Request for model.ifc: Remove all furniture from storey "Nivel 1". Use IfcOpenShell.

First a look at what the model holds.

```python
import ifcopenshell
import ifcopenshell.util.element

model = ifcopenshell.open("model.ifc")
print(model.schema)
storey = next(s for s in model.by_type("IfcBuildingStorey") if s.Name == "Nivel 1")
furniture = [e for e in ifcopenshell.util.element.get_decomposition(storey) if e.is_a("IfcFurnishingElement")]
seen = {}
for e in furniture:
    element_type = ifcopenshell.util.element.get_type(e)
    name = element_type.Name if element_type not in (None, e) else None
    seen[name] = seen.get(name, 0) + 1
for name, count in sorted(seen.items(), key=str):
    print(count, "x", name)
```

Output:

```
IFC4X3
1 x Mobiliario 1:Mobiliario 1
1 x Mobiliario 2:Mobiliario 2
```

```python
import ifcopenshell
import ifcopenshell.api.root
import ifcopenshell.util.element

model = ifcopenshell.open("model.ifc")

storey = next(s for s in model.by_type("IfcBuildingStorey") if s.Name == "Nivel 1")
furniture = [e for e in ifcopenshell.util.element.get_decomposition(storey) if e.is_a("IfcFurnishingElement")]

for e in furniture:
    ifcopenshell.api.root.remove_product(model, product=e)
print(len(furniture), "removed")

model.write("model_rev.ifc")
```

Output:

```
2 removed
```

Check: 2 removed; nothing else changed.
